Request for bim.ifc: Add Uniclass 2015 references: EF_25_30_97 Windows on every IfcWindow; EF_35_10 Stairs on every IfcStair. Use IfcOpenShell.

First a look at what the model holds.

```python
import ifcopenshell

model = ifcopenshell.open("bim.ifc")
print(model.schema)
print("classifications:", [c.Name for c in model.by_type("IfcClassification")])
for ifc_class in ("IfcDoor", "IfcRoof", "IfcStair", "IfcWall", "IfcWindow"):
    print(ifc_class, len(model.by_type(ifc_class)))
```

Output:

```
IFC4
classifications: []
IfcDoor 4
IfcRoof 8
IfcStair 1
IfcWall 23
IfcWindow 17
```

```python
import ifcopenshell
import ifcopenshell.api.classification

model = ifcopenshell.open("bim.ifc")

system = ifcopenshell.api.classification.add_classification(model, classification="Uniclass 2015")

codes = {
    "IfcWindow": ("EF_25_30_97", "Windows"),
    "IfcStair": ("EF_35_10", "Stairs"),
}
for ifc_class, (code, name) in codes.items():
    products = model.by_type(ifc_class)
    ifcopenshell.api.classification.add_reference(
        model, products=products, classification=system, identification=code, name=name
    )
    print(code, len(products))

model.write("bim_edited.ifc")
```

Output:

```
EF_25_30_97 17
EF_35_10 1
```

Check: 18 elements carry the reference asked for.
